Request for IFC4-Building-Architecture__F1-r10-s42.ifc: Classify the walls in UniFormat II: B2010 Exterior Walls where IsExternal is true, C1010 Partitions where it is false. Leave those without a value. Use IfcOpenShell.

First a look at what the model holds.

```python
import ifcopenshell
import ifcopenshell.util.element

model = ifcopenshell.open("IFC4-Building-Architecture__F1-r10-s42.ifc")
print(model.schema)
print("classifications:", [c.Name for c in model.by_type("IfcClassification")])
values = [ifcopenshell.util.element.get_pset(e, "Pset_WallCommon", "IsExternal") for e in model.by_type("IfcWall")]
for value in (True, False, None):
    print("IsExternal", value, values.count(value))
```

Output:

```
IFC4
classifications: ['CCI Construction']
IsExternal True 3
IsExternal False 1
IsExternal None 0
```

```python
import ifcopenshell
import ifcopenshell.api.classification
import ifcopenshell.util.element

model = ifcopenshell.open("IFC4-Building-Architecture__F1-r10-s42.ifc")

system = ifcopenshell.api.classification.add_classification(model, classification="UniFormat II")

walls = model.by_type("IfcWall")
external = {e: ifcopenshell.util.element.get_pset(e, "Pset_WallCommon", "IsExternal") for e in walls}
for flag, code, name in ((True, "B2010", "Exterior Walls"), (False, "C1010", "Partitions")):
    products = [e for e in walls if external[e] is flag]
    ifcopenshell.api.classification.add_reference(
        model, products=products, classification=system, identification=code, name=name
    )
    print(code, len(products))

model.write("IFC4-Building-Architecture__F1-r10-s42-out.ifc")
```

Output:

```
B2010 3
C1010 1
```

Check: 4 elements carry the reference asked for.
